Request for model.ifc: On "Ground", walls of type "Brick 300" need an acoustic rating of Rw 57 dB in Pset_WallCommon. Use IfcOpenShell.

First a look at what the model holds.

```python
import ifcopenshell
import ifcopenshell.util.element

model = ifcopenshell.open("model.ifc")
print(model.schema)
storey = next(s for s in model.by_type("IfcBuildingStorey") if s.Name == "Ground")
walls = [e for e in ifcopenshell.util.element.get_decomposition(storey) if e.is_a("IfcWall")]
seen = {}
for e in walls:
    element_type = ifcopenshell.util.element.get_type(e)
    key = (element_type.Name if element_type != e and element_type else None, ifcopenshell.util.element.get_pset(e, "Pset_WallCommon", "AcousticRating"))
    seen[key] = seen.get(key, 0) + 1
for (name, value), count in sorted(seen.items(), key=str):
    print(count, "x", name, "|", value)
```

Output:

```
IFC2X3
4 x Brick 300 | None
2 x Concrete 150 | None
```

```python
import ifcopenshell
import ifcopenshell.api.pset
import ifcopenshell.util.element

model = ifcopenshell.open("model.ifc")

storey = next(s for s in model.by_type("IfcBuildingStorey") if s.Name == "Ground")
walls = [e for e in ifcopenshell.util.element.get_decomposition(storey) if e.is_a("IfcWall")]

count = 0
for e in walls:
    element_type = ifcopenshell.util.element.get_type(e)
    if element_type in (None, e) or element_type.Name != "Brick 300":
        continue
    # add_pset returns the element's existing set when there is one.
    pset = ifcopenshell.api.pset.add_pset(model, product=e, name="Pset_WallCommon")
    ifcopenshell.api.pset.edit_pset(model, pset=pset, properties={"AcousticRating": "Rw 57 dB"})
    count += 1

print(count, "walls updated")

model.write("model_v2.ifc")
```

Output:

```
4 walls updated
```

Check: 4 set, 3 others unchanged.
